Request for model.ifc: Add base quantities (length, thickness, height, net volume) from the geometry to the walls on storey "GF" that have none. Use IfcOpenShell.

First a look at what the model holds.

```python
import ifcopenshell
import ifcopenshell.util.element
import ifcopenshell.util.unit

model = ifcopenshell.open("model.ifc")
print(model.schema)
for unit_type in ("LENGTHUNIT", "AREAUNIT", "VOLUMEUNIT"):
    print(unit_type, ifcopenshell.util.unit.calculate_unit_scale(model, unit_type))
storey = next(s for s in model.by_type("IfcBuildingStorey") if s.Name == "GF")
walls = [e for e in ifcopenshell.util.element.get_decomposition(storey) if e.is_a("IfcWall")]
for e in sorted(walls, key=lambda e: e.id()):
    print(e.id(), e.is_a(), e.Name, list(ifcopenshell.util.element.get_psets(e, qtos_only=True)), sep=" | ")
```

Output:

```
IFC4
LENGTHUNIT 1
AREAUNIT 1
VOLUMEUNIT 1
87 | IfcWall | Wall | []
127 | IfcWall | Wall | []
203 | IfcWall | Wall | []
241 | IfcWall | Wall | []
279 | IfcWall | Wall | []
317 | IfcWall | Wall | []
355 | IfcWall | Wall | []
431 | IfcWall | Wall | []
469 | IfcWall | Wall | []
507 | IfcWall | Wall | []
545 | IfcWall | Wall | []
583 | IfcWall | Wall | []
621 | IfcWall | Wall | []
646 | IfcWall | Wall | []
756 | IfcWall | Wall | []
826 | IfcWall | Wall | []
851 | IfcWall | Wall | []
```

```python
import ifcopenshell
import ifcopenshell.api.pset
import ifcopenshell.geom
import ifcopenshell.util.element
import ifcopenshell.util.shape
import ifcopenshell.util.unit

model = ifcopenshell.open("model.ifc")
unit_scale = ifcopenshell.util.unit.calculate_unit_scale(model)
volume_scale = ifcopenshell.util.unit.calculate_unit_scale(model, "VOLUMEUNIT")
settings = ifcopenshell.geom.settings()

storey = next(s for s in model.by_type("IfcBuildingStorey") if s.Name == "GF")
walls = [e for e in ifcopenshell.util.element.get_decomposition(storey) if e.is_a("IfcWall")]

for e in sorted(walls, key=lambda e: e.id()):
    if ifcopenshell.util.element.get_psets(e, qtos_only=True, should_inherit=False):
        continue
    # Geometry comes back in metres, in the element's own axes.
    shape = ifcopenshell.geom.create_shape(settings, e)
    values = {
        "Length": ifcopenshell.util.shape.get_x(shape.geometry) / unit_scale,
        "Width": ifcopenshell.util.shape.get_y(shape.geometry) / unit_scale,
        "Height": ifcopenshell.util.shape.get_z(shape.geometry) / unit_scale,
        "NetVolume": ifcopenshell.util.shape.get_volume(shape.geometry) / volume_scale,
    }
    qto = ifcopenshell.api.pset.add_qto(model, product=e, name="Qto_WallBaseQuantities")
    ifcopenshell.api.pset.edit_qto(model, qto=qto, properties=values)
    print(e.id(), {k: round(v, 3) for k, v in values.items()})

model.write("model_v2.ifc")
```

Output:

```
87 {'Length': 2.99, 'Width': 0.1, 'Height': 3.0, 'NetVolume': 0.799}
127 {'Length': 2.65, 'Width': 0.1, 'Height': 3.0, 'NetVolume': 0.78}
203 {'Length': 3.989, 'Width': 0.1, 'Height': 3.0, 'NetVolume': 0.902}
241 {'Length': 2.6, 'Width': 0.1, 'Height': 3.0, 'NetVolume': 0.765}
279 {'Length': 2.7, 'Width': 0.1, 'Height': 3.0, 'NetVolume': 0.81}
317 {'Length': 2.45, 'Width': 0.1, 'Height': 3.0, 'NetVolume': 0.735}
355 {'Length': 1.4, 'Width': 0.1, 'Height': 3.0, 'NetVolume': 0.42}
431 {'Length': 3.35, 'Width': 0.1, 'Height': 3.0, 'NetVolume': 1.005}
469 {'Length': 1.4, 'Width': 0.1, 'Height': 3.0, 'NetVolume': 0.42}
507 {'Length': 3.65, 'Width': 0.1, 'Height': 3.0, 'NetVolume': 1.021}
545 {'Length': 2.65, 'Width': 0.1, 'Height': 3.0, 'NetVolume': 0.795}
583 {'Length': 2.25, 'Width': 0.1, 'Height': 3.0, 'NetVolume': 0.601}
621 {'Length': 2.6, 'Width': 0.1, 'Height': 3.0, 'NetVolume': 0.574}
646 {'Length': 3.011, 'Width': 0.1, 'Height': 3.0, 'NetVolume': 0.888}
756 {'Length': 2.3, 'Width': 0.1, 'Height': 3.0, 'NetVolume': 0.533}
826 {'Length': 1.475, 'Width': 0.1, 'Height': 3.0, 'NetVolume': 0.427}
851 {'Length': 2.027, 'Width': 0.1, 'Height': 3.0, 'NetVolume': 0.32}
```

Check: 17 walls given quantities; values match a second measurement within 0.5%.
